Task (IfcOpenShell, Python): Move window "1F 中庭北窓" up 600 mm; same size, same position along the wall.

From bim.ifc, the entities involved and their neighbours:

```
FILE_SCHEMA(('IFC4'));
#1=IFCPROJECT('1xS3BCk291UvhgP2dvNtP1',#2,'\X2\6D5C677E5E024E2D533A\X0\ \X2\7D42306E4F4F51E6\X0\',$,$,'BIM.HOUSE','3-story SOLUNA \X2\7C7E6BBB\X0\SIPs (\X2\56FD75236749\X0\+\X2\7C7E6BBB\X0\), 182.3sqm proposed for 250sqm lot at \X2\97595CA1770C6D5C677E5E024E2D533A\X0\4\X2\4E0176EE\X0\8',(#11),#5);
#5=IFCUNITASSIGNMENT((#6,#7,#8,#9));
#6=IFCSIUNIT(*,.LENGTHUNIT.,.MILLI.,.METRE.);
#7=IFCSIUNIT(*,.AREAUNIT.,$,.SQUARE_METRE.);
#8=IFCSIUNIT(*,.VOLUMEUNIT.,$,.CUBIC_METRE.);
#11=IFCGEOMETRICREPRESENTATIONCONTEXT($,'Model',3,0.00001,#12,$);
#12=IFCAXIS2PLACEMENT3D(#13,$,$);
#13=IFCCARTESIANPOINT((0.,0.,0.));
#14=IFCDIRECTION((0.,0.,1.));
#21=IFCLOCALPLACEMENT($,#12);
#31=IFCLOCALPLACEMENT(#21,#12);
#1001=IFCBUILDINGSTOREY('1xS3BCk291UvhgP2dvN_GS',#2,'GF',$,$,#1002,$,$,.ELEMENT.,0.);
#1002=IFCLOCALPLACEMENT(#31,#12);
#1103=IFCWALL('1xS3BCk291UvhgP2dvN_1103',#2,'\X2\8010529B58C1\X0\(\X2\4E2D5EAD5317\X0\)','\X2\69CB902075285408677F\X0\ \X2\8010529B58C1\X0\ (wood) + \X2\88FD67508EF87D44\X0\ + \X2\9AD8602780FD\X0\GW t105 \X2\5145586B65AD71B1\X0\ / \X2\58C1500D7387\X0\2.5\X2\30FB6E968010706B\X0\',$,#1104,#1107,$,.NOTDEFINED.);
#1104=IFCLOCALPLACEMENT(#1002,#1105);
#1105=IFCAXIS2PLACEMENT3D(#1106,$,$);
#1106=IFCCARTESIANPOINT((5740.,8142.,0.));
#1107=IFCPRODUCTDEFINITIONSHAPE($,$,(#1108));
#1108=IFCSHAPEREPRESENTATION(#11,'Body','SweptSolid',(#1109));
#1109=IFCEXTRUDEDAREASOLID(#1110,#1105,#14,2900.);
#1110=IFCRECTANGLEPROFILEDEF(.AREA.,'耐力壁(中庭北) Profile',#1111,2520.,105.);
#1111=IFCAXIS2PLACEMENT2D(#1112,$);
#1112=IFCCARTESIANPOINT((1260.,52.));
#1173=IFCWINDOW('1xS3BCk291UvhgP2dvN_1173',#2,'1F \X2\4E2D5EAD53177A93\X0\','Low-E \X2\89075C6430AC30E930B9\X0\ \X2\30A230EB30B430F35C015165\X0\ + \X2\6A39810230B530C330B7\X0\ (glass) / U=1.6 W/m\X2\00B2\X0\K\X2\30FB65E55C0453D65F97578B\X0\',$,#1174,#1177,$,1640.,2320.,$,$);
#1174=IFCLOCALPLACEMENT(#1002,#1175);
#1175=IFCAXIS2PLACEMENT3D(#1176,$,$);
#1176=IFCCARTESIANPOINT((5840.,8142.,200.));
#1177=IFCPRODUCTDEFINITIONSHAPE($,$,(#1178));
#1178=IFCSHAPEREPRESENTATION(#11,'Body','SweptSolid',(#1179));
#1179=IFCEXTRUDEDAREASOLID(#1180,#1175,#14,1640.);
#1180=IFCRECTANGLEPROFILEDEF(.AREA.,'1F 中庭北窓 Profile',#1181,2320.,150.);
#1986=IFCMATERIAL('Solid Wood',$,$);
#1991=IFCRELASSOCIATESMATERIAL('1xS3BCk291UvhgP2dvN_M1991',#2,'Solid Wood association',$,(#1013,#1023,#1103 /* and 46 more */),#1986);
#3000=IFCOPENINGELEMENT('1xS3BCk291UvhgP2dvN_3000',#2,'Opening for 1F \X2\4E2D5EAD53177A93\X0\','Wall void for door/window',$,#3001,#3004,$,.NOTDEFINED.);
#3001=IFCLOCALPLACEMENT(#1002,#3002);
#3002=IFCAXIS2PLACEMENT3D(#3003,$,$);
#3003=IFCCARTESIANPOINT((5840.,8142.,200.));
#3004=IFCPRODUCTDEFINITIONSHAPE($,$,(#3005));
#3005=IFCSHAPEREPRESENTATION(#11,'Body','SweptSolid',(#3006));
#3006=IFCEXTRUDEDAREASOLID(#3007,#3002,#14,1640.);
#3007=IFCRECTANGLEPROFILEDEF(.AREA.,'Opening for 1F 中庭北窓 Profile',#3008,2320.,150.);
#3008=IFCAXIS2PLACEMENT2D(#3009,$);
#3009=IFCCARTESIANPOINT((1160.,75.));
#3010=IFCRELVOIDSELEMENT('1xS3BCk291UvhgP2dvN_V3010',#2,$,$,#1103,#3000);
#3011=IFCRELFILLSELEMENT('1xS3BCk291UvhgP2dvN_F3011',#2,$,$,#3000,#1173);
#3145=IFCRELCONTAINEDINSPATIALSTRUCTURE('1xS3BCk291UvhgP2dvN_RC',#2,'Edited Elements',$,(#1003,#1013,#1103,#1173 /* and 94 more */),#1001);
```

```python
import numpy as np
import ifcopenshell
import ifcopenshell.api.geometry
import ifcopenshell.util.placement
import ifcopenshell.util.unit

model = ifcopenshell.open("bim.ifc")
unit_scale = ifcopenshell.util.unit.calculate_unit_scale(model)

window = model.by_guid("1xS3BCk291UvhgP2dvN_1173")
opening = window.FillsVoids[0].RelatingOpeningElement
dz = 600.0

shift = np.array([0.0, 0.0, dz])
# The window is not placed relative to its opening, so move both.
for product in (opening, window):
    matrix = ifcopenshell.util.placement.get_local_placement(product.ObjectPlacement)
    matrix[:3, 3] += shift
    ifcopenshell.api.geometry.edit_object_placement(model, product=product, matrix=matrix, is_si=False)

print(f"moved by {dz * unit_scale:+.3f} m")

model.write("bim_v2.ifc")
```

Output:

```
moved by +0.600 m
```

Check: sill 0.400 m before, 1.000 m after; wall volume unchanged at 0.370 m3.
